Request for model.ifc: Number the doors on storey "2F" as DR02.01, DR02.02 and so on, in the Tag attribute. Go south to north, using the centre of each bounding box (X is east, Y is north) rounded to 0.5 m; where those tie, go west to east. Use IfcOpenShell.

First a look at what the model holds.

```python
import ifcopenshell
import ifcopenshell.util.element
import ifcopenshell.util.placement

model = ifcopenshell.open("model.ifc")
print(model.schema)
storey = next(s for s in model.by_type("IfcBuildingStorey") if s.Name == "2F")
doors = [e for e in ifcopenshell.util.element.get_decomposition(storey) if e.is_a("IfcDoor")]
for e in sorted(doors, key=lambda e: e.id()):
    origin = ifcopenshell.util.placement.get_local_placement(e.ObjectPlacement)[:3, 3]
    print(e.id(), e.Tag, e.Name, origin.round(2) + 0.0, sep=" | ")
```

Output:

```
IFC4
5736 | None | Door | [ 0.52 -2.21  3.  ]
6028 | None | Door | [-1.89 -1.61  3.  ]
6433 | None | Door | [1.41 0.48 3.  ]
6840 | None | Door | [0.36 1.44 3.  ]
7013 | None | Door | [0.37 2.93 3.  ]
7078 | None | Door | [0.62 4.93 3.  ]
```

```python
import ifcopenshell
import ifcopenshell.geom
import ifcopenshell.util.element
import ifcopenshell.util.shape

model = ifcopenshell.open("model.ifc")
settings = ifcopenshell.geom.settings()
settings.set("use-world-coords", True)


def centre(element):
    shape = ifcopenshell.geom.create_shape(settings, element)
    return ifcopenshell.util.shape.get_bbox_centroid(shape.geometry)


storey = next(s for s in model.by_type("IfcBuildingStorey") if s.Name == "2F")
doors = [e for e in ifcopenshell.util.element.get_decomposition(storey) if e.is_a("IfcDoor")]

# Insertion points can sit at a corner or the storey origin, so sort by the geometry (in metres).
centres = {e: centre(e) for e in doors}
doors.sort(key=lambda e: (round(centres[e][1] / 0.5), centres[e][0]))

for i, e in enumerate(doors, start=1):
    number = f"DR02.{i:02d}"
    e.Tag = number
    print(e.id(), number)

model.write("model-out.ifc")
```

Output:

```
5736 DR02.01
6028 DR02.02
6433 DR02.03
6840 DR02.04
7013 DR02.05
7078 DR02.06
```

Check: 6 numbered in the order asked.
